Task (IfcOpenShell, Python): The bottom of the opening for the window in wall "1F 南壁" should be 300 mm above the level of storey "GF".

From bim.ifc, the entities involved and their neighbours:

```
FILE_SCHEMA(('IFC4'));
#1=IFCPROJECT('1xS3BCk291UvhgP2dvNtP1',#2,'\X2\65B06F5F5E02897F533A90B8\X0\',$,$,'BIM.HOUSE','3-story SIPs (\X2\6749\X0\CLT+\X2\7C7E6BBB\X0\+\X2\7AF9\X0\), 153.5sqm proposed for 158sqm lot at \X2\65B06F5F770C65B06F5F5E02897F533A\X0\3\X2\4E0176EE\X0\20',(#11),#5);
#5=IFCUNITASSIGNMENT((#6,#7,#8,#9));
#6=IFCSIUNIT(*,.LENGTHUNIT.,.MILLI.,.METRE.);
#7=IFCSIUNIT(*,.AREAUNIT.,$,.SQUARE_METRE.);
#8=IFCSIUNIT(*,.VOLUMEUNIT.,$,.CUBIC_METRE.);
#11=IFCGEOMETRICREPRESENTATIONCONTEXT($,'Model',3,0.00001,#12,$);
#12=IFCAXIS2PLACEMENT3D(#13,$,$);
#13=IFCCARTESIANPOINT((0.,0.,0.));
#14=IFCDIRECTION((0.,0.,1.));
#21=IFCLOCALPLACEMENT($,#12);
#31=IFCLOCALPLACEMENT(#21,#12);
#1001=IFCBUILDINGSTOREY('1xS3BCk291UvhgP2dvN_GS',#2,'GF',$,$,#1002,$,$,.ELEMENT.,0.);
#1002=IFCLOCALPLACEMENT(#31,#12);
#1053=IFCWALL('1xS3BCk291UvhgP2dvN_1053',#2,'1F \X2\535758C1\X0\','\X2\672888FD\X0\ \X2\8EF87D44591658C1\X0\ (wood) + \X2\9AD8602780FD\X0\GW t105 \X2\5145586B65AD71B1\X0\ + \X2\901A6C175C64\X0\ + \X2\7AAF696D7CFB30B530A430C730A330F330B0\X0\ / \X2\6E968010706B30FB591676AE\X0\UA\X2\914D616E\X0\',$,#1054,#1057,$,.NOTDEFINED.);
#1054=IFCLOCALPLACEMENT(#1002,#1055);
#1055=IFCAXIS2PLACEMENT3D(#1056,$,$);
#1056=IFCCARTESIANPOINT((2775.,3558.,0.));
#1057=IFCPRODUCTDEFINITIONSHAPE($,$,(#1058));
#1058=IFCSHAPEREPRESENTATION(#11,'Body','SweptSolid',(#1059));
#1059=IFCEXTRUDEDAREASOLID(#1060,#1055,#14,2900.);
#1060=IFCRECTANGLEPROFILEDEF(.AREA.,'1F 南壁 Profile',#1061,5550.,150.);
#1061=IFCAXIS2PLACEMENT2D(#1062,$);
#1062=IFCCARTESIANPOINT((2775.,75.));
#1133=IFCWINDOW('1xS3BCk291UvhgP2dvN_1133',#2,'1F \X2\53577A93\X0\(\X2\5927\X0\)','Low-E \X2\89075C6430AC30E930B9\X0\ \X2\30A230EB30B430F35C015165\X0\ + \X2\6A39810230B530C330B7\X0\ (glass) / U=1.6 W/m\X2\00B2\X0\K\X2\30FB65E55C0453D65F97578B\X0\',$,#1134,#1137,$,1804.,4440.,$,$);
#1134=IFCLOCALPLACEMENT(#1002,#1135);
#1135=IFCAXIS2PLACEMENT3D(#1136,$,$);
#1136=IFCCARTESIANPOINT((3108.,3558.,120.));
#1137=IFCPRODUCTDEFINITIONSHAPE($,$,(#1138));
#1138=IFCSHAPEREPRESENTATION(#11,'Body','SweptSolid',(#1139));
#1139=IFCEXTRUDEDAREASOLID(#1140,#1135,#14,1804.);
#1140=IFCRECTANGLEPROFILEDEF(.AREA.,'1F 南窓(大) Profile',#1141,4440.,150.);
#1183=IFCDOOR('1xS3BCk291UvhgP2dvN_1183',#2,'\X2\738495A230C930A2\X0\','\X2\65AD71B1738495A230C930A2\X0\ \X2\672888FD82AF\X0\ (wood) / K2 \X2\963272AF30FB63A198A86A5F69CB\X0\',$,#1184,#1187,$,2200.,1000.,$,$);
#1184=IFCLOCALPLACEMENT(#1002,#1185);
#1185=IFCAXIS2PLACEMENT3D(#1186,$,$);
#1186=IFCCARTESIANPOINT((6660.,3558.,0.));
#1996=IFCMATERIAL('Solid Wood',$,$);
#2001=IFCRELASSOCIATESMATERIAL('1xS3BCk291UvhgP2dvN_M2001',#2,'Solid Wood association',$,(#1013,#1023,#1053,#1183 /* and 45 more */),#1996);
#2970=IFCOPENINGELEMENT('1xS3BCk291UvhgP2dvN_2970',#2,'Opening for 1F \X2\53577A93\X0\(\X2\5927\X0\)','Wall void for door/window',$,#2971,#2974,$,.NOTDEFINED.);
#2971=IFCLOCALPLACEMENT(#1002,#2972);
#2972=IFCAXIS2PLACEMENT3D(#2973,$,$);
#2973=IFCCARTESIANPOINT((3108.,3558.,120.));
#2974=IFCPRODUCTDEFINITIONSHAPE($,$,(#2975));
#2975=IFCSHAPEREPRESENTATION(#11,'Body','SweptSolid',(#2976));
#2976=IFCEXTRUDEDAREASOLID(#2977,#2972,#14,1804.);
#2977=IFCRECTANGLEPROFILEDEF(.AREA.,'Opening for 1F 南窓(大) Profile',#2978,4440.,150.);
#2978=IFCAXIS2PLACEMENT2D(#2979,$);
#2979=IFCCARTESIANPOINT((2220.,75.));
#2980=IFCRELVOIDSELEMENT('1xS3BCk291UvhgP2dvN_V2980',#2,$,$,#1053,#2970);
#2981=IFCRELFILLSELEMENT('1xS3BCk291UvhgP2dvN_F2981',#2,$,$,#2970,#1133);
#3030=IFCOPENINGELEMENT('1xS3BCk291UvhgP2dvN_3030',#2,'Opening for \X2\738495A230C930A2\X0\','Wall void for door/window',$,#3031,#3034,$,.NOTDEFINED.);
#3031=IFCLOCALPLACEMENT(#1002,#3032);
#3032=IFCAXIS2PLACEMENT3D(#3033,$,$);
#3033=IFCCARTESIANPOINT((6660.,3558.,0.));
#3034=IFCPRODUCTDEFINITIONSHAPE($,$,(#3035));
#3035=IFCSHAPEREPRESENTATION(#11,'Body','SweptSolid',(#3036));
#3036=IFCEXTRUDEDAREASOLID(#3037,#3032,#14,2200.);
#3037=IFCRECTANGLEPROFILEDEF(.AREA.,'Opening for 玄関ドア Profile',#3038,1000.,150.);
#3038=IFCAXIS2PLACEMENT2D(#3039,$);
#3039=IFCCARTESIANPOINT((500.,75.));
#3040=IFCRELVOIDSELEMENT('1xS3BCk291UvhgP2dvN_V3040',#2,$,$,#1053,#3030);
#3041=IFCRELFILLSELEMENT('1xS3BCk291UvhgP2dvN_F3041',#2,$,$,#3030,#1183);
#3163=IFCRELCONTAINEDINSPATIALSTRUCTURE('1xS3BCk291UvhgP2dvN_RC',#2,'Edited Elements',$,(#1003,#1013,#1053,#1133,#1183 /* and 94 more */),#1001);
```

```python
import numpy as np
import ifcopenshell
import ifcopenshell.api.geometry
import ifcopenshell.geom
import ifcopenshell.util.element
import ifcopenshell.util.placement
import ifcopenshell.util.shape
import ifcopenshell.util.unit

model = ifcopenshell.open("bim.ifc")
unit_scale = ifcopenshell.util.unit.calculate_unit_scale(model)

window = model.by_id(1133)
opening = window.FillsVoids[0].RelatingOpeningElement
storey = ifcopenshell.util.element.get_container(window, ifc_class="IfcBuildingStorey")
level = ifcopenshell.util.placement.get_local_placement(storey.ObjectPlacement)[2, 3]

# The opening's origin need not be at the sill, so measure its lowest point.
shape = ifcopenshell.geom.create_shape(ifcopenshell.geom.settings(), opening)
bottom = ifcopenshell.util.shape.get_shape_bottom_elevation(shape, shape.geometry) / unit_scale
dz = level + 300.0 - bottom

shift = np.array([0.0, 0.0, dz])
# The window is not placed relative to its opening, so move both.
for product in (opening, window):
    matrix = ifcopenshell.util.placement.get_local_placement(product.ObjectPlacement)
    matrix[:3, 3] += shift
    ifcopenshell.api.geometry.edit_object_placement(model, product=product, matrix=matrix, is_si=False)

print(f"moved by {dz * unit_scale:+.3f} m")

model.write("bim_edited.ifc")
```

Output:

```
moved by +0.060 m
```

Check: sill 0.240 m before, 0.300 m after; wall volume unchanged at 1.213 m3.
